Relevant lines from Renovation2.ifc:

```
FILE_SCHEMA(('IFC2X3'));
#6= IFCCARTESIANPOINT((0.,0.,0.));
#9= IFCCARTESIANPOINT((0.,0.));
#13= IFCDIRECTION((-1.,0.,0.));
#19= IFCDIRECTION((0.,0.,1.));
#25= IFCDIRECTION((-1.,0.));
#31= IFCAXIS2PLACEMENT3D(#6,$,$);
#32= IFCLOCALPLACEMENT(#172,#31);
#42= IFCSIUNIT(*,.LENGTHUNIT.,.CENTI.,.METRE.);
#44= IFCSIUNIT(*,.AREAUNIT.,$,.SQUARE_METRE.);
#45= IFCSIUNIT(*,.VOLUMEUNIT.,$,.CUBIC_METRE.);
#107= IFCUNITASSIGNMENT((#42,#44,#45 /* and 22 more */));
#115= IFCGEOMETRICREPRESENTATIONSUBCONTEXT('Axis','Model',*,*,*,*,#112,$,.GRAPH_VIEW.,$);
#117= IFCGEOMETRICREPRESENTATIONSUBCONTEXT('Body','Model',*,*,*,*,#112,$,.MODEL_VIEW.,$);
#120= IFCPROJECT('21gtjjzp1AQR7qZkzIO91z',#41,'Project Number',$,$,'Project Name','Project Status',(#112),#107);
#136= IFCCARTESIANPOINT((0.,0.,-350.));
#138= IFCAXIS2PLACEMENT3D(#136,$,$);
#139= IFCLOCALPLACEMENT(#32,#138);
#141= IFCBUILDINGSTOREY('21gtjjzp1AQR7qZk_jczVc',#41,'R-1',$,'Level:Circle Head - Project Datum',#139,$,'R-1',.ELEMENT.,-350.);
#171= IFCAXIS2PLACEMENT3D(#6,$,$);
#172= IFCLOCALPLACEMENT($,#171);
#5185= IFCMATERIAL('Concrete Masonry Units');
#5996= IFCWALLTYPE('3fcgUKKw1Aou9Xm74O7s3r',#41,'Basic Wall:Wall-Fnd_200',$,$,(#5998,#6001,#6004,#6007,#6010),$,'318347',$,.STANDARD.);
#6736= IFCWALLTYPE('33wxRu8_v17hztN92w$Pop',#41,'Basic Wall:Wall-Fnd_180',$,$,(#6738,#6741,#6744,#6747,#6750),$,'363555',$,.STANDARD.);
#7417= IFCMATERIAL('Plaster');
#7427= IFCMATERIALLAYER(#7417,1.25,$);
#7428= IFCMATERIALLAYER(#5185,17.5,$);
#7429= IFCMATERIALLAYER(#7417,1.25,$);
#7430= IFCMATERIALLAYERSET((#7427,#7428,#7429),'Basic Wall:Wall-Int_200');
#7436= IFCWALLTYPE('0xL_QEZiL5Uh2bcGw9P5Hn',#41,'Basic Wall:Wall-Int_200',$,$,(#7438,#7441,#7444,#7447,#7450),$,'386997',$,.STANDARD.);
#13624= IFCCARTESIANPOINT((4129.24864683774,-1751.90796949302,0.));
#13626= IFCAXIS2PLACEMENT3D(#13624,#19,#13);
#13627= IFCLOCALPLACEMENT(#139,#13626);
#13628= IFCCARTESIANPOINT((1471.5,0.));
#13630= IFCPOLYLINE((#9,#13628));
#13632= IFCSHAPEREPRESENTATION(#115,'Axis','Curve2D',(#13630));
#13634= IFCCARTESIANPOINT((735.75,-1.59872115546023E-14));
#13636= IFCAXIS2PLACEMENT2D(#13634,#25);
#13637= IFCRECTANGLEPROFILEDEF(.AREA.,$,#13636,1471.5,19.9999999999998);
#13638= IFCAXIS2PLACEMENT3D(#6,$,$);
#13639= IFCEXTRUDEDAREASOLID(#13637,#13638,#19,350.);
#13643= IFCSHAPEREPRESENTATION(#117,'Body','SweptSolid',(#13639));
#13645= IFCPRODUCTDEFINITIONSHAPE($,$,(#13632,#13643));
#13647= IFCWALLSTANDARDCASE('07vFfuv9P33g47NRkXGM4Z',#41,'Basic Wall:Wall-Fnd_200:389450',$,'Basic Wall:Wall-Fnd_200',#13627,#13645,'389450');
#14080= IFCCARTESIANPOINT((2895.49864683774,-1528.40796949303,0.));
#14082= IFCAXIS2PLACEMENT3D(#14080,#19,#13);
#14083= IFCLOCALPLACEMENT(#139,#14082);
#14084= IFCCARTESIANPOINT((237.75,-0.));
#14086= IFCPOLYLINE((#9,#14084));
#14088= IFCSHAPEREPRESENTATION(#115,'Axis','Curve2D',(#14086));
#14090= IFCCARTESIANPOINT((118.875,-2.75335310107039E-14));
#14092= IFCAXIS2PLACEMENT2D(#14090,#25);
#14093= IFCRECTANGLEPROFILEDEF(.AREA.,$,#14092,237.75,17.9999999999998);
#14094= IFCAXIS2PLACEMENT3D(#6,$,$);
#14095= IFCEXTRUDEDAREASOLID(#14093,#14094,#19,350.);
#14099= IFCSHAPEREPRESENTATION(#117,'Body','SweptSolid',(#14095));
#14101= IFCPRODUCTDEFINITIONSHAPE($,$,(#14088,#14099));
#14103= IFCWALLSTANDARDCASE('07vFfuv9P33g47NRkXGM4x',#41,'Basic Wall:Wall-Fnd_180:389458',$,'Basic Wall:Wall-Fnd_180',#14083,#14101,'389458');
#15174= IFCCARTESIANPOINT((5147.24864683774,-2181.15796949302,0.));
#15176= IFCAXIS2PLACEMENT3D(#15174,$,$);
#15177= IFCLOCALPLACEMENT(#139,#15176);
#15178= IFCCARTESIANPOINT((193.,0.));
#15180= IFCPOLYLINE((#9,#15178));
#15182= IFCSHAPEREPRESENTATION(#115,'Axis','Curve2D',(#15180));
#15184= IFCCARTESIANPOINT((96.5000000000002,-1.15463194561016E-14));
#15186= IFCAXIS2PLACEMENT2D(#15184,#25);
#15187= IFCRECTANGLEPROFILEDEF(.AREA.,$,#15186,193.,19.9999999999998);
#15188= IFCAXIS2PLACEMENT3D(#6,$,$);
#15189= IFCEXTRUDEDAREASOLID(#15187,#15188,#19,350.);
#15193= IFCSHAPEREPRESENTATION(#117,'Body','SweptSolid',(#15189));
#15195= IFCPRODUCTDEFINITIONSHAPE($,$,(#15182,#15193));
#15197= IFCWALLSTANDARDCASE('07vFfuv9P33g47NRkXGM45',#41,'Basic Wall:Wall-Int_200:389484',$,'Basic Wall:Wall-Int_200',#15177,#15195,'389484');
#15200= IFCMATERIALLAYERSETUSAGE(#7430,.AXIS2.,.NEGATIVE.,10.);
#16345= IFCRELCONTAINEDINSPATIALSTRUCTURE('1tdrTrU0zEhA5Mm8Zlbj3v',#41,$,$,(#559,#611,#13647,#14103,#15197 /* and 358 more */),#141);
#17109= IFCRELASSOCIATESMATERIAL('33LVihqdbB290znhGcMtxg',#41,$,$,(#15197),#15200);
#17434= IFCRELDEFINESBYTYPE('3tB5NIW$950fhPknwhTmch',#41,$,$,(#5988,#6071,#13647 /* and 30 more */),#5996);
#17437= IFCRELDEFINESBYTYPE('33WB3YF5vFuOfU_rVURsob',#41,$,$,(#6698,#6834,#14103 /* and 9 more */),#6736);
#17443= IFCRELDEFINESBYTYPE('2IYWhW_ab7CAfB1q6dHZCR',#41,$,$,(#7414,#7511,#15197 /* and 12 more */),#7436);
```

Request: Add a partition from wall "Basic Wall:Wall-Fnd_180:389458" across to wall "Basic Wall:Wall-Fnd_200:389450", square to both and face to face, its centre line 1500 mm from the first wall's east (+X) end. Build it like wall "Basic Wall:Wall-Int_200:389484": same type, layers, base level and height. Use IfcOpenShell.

```python
import numpy as np
import ifcopenshell
import ifcopenshell.api.geometry
import ifcopenshell.api.material
import ifcopenshell.api.pset
import ifcopenshell.api.root
import ifcopenshell.api.spatial
import ifcopenshell.api.type
import ifcopenshell.geom
import ifcopenshell.util.element
import ifcopenshell.util.placement
import ifcopenshell.util.representation
import ifcopenshell.util.shape
import ifcopenshell.util.unit

model = ifcopenshell.open("Renovation2.ifc")
unit_scale = ifcopenshell.util.unit.calculate_unit_scale(model)
settings = ifcopenshell.geom.settings()
settings.set("use-world-coords", True)

start_wall = model.by_guid("07vFfuv9P33g47NRkXGM4x")
end_wall = model.by_id(13647)
like = model.by_guid("07vFfuv9P33g47NRkXGM45")
matrix = ifcopenshell.util.placement.get_local_placement(start_wall.ObjectPlacement)
matrix[:3, 3] *= unit_scale


def extent(element):
    """Bounding box in the first wall's axes, in metres."""
    shape = ifcopenshell.geom.create_shape(settings, element)
    points = (ifcopenshell.util.shape.get_vertices(shape.geometry) - matrix[:3, 3]) @ matrix[:3, :3]
    return points.min(axis=0), points.max(axis=0)


y_start = extent(start_wall)[1][1]
y_end = extent(end_wall)[0][1]
like_min, like_max = extent(like)
length, height = float(abs(y_end - y_start)), float(like_max[2] - like_min[2])
layer_set = ifcopenshell.util.element.get_material(like, should_skip_usage=True)
thickness = sum(layer.LayerThickness for layer in layer_set.MaterialLayers) * unit_scale

wall = ifcopenshell.api.root.create_entity(model, ifc_class="IfcWallStandardCase", name="New partition")
storey = ifcopenshell.util.element.get_container(like)
ifcopenshell.api.spatial.assign_container(model, products=[wall], relating_structure=storey)
ifcopenshell.api.type.assign_type(
    model, related_objects=[wall], relating_type=ifcopenshell.util.element.get_type(like), should_map_representations=False
)
rel = ifcopenshell.api.material.assign_material(
    model, products=[wall], type="IfcMaterialLayerSetUsage", material=layer_set
)
rel.RelatingMaterial.OffsetFromReferenceLine = -thickness / 2 / unit_scale
pset = ifcopenshell.api.pset.add_pset(model, product=wall, name="Pset_WallCommon")
ifcopenshell.api.pset.edit_pset(model, pset=pset, properties={"IsExternal": False, "LoadBearing": False})

# The axis runs down the middle of the wall.
axis = ifcopenshell.api.geometry.add_axis_representation(
    model, context=ifcopenshell.util.representation.get_context(model, "Model", "Axis"), axis=[(0.0, 0.0), (length, 0.0)]
)
body = ifcopenshell.api.geometry.add_wall_representation(
    model,
    context=ifcopenshell.util.representation.get_context(model, "Model", "Body", "MODEL_VIEW"),
    length=length,
    height=height,
    thickness=thickness,
    offset=-thickness / 2,
)
for representation in (axis, body):
    ifcopenshell.api.geometry.assign_representation(model, product=wall, representation=representation)

placement = matrix @ ifcopenshell.util.placement.rotation(90, "Z")
placement[:, 3] = matrix @ np.array([extent(start_wall)[0][0] + 1.5, y_start, like_min[2], 1.0])
ifcopenshell.api.geometry.edit_object_placement(model, product=wall, matrix=placement)

print(f"partition {length:.3f} m long, {height:.3f} m high, {thickness:.3f} m thick")

model.write("Renovation2_v2.ifc")
```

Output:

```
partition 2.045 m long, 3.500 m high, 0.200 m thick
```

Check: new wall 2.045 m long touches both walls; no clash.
